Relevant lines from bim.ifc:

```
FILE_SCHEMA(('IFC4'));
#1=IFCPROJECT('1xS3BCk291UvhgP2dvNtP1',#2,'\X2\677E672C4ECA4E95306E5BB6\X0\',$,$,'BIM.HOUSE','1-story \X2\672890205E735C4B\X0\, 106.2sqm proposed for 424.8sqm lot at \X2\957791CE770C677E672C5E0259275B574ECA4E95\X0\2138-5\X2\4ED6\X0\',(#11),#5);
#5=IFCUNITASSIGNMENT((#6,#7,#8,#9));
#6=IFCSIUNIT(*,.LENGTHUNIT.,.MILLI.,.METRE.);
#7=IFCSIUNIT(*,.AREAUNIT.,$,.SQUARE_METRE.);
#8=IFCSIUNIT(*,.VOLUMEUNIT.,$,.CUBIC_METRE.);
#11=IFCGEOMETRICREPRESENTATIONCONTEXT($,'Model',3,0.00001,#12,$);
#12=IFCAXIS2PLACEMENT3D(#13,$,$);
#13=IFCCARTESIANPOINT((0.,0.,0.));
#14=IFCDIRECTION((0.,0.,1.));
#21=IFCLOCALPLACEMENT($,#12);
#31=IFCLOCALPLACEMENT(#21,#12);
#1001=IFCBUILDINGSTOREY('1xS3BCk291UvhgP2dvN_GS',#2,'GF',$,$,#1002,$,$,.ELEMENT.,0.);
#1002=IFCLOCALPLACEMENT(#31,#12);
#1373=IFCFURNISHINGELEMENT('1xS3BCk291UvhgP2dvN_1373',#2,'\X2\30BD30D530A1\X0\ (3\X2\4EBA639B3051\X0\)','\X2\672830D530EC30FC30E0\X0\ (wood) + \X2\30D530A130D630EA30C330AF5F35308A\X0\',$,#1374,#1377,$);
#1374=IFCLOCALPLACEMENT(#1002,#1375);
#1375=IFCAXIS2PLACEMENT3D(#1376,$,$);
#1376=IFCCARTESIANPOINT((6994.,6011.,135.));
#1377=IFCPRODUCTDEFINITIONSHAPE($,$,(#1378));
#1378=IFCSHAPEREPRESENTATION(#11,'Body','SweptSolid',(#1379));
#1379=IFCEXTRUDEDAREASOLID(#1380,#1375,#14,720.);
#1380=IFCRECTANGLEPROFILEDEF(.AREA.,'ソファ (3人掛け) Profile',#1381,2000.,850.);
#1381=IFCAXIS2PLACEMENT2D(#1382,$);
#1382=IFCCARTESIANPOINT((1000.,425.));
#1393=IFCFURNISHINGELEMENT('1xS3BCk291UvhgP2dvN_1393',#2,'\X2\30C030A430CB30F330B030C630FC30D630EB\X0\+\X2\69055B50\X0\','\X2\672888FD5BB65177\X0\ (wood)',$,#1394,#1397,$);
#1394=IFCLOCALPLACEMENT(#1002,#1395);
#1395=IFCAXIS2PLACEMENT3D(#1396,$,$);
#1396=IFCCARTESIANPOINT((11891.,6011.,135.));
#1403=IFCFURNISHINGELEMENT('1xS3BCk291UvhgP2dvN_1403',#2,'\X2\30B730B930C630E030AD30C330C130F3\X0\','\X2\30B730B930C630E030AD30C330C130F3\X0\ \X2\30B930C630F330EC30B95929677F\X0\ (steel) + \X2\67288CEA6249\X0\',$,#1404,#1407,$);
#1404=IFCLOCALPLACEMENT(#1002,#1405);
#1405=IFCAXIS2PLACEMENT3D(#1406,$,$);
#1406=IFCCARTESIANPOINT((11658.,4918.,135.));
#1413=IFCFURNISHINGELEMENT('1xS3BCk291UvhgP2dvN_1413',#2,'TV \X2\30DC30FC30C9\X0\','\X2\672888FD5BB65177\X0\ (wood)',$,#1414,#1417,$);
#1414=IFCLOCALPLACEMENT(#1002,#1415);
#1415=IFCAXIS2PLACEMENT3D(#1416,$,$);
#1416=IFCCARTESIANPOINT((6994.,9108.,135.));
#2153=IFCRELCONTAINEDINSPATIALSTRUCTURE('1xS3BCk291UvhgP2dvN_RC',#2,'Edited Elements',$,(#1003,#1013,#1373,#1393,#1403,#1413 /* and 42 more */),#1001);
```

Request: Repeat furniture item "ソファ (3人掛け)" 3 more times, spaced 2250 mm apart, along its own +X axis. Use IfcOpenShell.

```python
import ifcopenshell
import ifcopenshell.api.geometry
import ifcopenshell.api.root
import ifcopenshell.util.element
import ifcopenshell.util.placement
import ifcopenshell.util.unit

model = ifcopenshell.open("bim.ifc")
unit_scale = ifcopenshell.util.unit.calculate_unit_scale(model)


def reuse_history(source, copy):
    """copy_class also copies each property set's owner history, people and application; keep the originals."""
    for rel in copy.IsDefinedBy:
        if rel.is_a("IfcRelDefinesByProperties") and (history := rel.RelatingPropertyDefinition.OwnerHistory):
            rel.RelatingPropertyDefinition.OwnerHistory = source.OwnerHistory
            ifcopenshell.util.element.remove_deep2(model, history)


source = model.by_id(1373)
base = ifcopenshell.util.placement.get_local_placement(source.ObjectPlacement)
step = base[:3, 0] * 2.25 / unit_scale

for i in range(1, 4):
    copy = ifcopenshell.api.root.copy_class(model, product=source)
    copy.Representation = ifcopenshell.util.element.copy_deep(
        model, source.Representation, exclude=["IfcGeometricRepresentationContext", "IfcRepresentationMap"]
    )
    reuse_history(source, copy)
    matrix = base.copy()
    matrix[:3, 3] += i * step
    print("added at", matrix[:3, 3].round(3) + 0.0)
    ifcopenshell.api.geometry.edit_object_placement(model, product=copy, matrix=matrix, is_si=False)

model.write("bim-out.ifc")
```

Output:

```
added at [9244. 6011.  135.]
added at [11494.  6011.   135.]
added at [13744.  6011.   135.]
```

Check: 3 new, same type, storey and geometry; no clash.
